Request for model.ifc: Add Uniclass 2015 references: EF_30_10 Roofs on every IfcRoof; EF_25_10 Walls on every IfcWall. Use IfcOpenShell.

First a look at what the model holds.

```python
import ifcopenshell

model = ifcopenshell.open("model.ifc")
print(model.schema)
print("classifications:", [c.Name for c in model.by_type("IfcClassification")])
for ifc_class in ("IfcDoor", "IfcRoof", "IfcStair", "IfcWall", "IfcWindow"):
    print(ifc_class, len(model.by_type(ifc_class)))
```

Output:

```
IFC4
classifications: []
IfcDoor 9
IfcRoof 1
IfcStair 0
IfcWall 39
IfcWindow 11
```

```python
import ifcopenshell
import ifcopenshell.api.classification

model = ifcopenshell.open("model.ifc")

system = ifcopenshell.api.classification.add_classification(model, classification="Uniclass 2015")

codes = {
    "IfcRoof": ("EF_30_10", "Roofs"),
    "IfcWall": ("EF_25_10", "Walls"),
}
for ifc_class, (code, name) in codes.items():
    products = model.by_type(ifc_class)
    ifcopenshell.api.classification.add_reference(
        model, products=products, classification=system, identification=code, name=name
    )
    print(code, len(products))

model.write("model-out.ifc")
```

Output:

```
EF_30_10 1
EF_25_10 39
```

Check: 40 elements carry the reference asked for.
